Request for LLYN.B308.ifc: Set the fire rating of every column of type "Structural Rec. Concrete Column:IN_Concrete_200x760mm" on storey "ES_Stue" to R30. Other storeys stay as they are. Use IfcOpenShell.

First a look at what the model holds.

```python
import ifcopenshell
import ifcopenshell.util.element

model = ifcopenshell.open("LLYN.B308.ifc")
print(model.schema)
storey = next(s for s in model.by_type("IfcBuildingStorey") if s.Name == "ES_Stue")
columns = [e for e in ifcopenshell.util.element.get_decomposition(storey) if e.is_a("IfcColumn")]
seen = {}
for e in columns:
    element_type = ifcopenshell.util.element.get_type(e)
    key = (element_type.Name if element_type != e and element_type else None, ifcopenshell.util.element.get_pset(e, "Pset_ColumnCommon", "FireRating"))
    seen[key] = seen.get(key, 0) + 1
for (name, value), count in sorted(seen.items(), key=str):
    print(count, "x", name, "|", value)
```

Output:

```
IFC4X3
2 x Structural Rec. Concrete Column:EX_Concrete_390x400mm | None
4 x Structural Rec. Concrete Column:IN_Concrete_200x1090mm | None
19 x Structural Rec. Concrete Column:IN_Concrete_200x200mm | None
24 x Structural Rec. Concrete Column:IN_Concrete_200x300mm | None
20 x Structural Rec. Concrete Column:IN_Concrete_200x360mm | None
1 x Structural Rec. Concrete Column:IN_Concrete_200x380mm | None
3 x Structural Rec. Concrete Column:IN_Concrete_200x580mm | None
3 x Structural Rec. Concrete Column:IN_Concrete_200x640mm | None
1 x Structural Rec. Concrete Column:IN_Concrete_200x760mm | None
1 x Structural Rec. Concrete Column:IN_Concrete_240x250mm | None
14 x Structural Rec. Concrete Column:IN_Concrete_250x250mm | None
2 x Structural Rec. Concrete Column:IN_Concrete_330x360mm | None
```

```python
import ifcopenshell
import ifcopenshell.api.pset
import ifcopenshell.util.element

model = ifcopenshell.open("LLYN.B308.ifc")

storey = next(s for s in model.by_type("IfcBuildingStorey") if s.Name == "ES_Stue")
columns = [e for e in ifcopenshell.util.element.get_decomposition(storey) if e.is_a("IfcColumn")]

count = 0
for e in columns:
    element_type = ifcopenshell.util.element.get_type(e)
    if element_type in (None, e) or element_type.Name != "Structural Rec. Concrete Column:IN_Concrete_200x760mm":
        continue
    # add_pset returns the element's existing set when there is one.
    pset = ifcopenshell.api.pset.add_pset(model, product=e, name="Pset_ColumnCommon")
    ifcopenshell.api.pset.edit_pset(model, pset=pset, properties={"FireRating": "R30"})
    count += 1

print(count, "columns updated")

model.write("LLYN.B308_updated.ifc")
```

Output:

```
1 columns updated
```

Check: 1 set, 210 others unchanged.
